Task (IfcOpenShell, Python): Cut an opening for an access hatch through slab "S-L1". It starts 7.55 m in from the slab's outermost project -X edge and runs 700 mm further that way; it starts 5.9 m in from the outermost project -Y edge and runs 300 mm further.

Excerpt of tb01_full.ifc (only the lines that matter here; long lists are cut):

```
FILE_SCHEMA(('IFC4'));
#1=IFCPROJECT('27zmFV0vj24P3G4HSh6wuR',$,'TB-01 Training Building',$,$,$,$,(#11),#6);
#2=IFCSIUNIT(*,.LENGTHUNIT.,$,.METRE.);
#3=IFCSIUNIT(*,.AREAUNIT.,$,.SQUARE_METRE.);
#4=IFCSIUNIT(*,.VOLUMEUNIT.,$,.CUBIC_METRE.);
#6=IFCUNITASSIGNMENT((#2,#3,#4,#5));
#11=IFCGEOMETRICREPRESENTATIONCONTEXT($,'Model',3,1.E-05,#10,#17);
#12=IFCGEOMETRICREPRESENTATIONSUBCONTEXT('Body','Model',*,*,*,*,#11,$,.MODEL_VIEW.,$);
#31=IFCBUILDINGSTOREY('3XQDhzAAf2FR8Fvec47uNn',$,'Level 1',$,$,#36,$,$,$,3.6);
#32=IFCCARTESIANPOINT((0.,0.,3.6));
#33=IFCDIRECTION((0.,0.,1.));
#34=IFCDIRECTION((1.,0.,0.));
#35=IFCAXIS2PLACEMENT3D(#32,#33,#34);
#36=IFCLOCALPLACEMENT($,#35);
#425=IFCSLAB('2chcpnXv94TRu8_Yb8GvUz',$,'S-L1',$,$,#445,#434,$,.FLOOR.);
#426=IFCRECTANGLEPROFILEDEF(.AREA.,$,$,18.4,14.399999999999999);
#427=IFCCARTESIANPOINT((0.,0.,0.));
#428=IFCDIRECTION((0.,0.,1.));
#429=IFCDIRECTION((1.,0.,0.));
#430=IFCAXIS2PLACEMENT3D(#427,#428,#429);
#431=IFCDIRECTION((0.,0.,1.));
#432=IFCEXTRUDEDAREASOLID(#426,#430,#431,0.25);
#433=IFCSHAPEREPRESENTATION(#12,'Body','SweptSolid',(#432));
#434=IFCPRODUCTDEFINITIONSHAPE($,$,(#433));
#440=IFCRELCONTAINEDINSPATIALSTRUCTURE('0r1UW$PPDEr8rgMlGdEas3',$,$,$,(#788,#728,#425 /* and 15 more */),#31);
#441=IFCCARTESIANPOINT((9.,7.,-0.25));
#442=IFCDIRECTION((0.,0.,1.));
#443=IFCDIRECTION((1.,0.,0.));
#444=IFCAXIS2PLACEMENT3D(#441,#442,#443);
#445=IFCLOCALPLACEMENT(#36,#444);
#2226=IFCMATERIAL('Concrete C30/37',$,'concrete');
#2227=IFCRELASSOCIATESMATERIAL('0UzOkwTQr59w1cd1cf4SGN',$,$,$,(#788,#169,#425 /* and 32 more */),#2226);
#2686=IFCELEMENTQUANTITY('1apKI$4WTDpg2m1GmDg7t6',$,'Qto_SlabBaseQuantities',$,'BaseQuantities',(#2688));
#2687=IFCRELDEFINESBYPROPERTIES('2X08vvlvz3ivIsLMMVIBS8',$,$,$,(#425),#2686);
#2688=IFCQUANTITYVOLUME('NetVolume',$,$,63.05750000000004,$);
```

```python
import numpy as np
import ifcopenshell
import ifcopenshell.api.feature
import ifcopenshell.api.geometry
import ifcopenshell.api.pset
import ifcopenshell.api.root
import ifcopenshell.geom
import ifcopenshell.util.element
import ifcopenshell.util.placement
import ifcopenshell.util.representation
import ifcopenshell.util.shape
import ifcopenshell.util.unit

model = ifcopenshell.open("tb01_full.ifc")
unit_scale = ifcopenshell.util.unit.calculate_unit_scale(model)
volume_scale = ifcopenshell.util.unit.calculate_unit_scale(model, "VOLUMEUNIT")
settings = ifcopenshell.geom.settings()


def volume(element):
    """Net volume in cubic metres, openings subtracted."""
    shape = ifcopenshell.geom.create_shape(settings, element)
    return ifcopenshell.util.shape.get_volume(shape.geometry)


slab = model.by_id(425)
before = volume(slab)

# Extent in the slab's own axes, in metres. The edges named are its -X and -Y sides.
slab_shape = ifcopenshell.geom.create_shape(settings, slab)
vertices = ifcopenshell.util.shape.get_vertices(slab_shape.geometry)
x_min, y_min, bottom = vertices.min(axis=0)
top = vertices[:, 2].max()

opening = ifcopenshell.api.root.create_entity(model, ifc_class="IfcOpeningElement", name="Access hatch opening", predefined_type="OPENING")
context = ifcopenshell.util.representation.get_context(model, "Model", "Body", "MODEL_VIEW")
width, depth = 0.7, 0.3
outline = [(0.0, 0.0), (width, 0.0), (width, depth), (0.0, depth), (0.0, 0.0)]
# Overshoot both faces by 50 mm so the cut is clean.
shape = ifcopenshell.api.geometry.add_slab_representation(
    model, context=context, depth=top - bottom + 0.1, polyline=outline
)
ifcopenshell.api.geometry.assign_representation(model, product=opening, representation=shape)

matrix = ifcopenshell.util.placement.get_local_placement(slab.ObjectPlacement)
matrix[:, 3] = matrix @ np.append(np.array([x_min + 7.55, y_min + 5.9, bottom - 0.05]) / unit_scale, 1.0)
ifcopenshell.api.geometry.edit_object_placement(model, product=opening, matrix=matrix, is_si=False)
ifcopenshell.api.feature.add_feature(model, feature=opening, element=slab)

after = volume(slab)

# Update the slab's stored quantities.
qto = model.by_id(ifcopenshell.util.element.get_pset(slab, "Qto_SlabBaseQuantities", should_inherit=False)["id"])
ifcopenshell.api.pset.edit_qto(model, qto=qto, properties={"NetVolume": after / volume_scale})

print(f"slab volume {before:.3f} -> {after:.3f} m3")

model.write("tb01_full_updated.ifc")
```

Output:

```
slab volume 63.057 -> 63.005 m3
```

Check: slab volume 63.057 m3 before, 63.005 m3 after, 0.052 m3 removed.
